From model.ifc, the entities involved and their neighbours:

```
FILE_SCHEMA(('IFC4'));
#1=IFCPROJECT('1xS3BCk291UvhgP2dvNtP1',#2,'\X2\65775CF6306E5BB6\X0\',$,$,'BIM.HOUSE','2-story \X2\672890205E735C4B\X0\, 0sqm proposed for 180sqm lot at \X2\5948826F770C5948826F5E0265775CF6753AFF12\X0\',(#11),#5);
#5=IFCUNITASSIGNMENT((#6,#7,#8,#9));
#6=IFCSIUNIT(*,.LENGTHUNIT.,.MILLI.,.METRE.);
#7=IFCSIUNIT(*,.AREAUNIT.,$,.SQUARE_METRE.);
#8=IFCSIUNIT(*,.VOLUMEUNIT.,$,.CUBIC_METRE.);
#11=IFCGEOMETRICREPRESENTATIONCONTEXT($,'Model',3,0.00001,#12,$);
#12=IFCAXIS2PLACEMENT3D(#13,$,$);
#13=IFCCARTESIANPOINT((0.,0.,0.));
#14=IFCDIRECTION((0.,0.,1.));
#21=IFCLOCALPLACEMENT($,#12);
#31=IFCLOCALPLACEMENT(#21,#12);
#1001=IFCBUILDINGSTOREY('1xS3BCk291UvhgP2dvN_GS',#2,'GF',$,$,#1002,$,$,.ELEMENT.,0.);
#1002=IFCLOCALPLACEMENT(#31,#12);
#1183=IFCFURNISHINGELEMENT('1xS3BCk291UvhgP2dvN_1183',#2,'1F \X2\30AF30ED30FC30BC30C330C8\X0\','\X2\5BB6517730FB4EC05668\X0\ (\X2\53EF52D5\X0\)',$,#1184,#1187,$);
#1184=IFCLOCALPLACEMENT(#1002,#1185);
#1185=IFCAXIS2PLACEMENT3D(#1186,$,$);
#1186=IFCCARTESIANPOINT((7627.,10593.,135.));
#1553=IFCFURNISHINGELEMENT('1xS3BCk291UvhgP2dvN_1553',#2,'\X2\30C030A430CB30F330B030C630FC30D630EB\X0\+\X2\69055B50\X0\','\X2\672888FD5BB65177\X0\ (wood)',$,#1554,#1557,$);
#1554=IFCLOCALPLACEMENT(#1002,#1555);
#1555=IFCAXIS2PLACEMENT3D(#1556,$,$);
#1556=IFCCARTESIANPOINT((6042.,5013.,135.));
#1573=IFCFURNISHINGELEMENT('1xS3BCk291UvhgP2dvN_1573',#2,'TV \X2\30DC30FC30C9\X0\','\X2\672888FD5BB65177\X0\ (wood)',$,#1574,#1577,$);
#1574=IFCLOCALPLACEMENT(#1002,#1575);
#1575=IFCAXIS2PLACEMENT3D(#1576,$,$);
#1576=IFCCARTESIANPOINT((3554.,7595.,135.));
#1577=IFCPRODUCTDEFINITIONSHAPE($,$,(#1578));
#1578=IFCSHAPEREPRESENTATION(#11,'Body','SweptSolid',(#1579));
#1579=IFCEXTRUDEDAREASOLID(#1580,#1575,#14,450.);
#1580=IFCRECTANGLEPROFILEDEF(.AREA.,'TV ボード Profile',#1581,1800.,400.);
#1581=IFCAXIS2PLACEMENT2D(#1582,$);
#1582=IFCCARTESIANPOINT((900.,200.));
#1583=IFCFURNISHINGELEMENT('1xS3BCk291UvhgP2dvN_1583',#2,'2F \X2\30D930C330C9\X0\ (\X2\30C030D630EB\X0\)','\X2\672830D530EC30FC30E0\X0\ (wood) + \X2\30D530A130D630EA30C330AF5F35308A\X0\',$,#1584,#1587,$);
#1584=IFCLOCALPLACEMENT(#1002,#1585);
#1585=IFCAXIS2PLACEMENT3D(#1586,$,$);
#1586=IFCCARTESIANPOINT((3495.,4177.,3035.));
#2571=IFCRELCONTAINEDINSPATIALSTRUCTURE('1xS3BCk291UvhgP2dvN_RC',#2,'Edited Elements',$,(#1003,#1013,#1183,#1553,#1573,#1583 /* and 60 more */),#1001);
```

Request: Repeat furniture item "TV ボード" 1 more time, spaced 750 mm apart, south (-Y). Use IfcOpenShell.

```python
import numpy as np
import ifcopenshell
import ifcopenshell.api.geometry
import ifcopenshell.api.root
import ifcopenshell.util.element
import ifcopenshell.util.placement

model = ifcopenshell.open("model.ifc")


def reuse_history(source, copy):
    """copy_class also copies each property set's owner history, people and application; keep the originals."""
    for rel in copy.IsDefinedBy:
        if rel.is_a("IfcRelDefinesByProperties") and (history := rel.RelatingPropertyDefinition.OwnerHistory):
            rel.RelatingPropertyDefinition.OwnerHistory = source.OwnerHistory
            ifcopenshell.util.element.remove_deep2(model, history)


source = model.by_guid("1xS3BCk291UvhgP2dvN_1573")
base = ifcopenshell.util.placement.get_local_placement(source.ObjectPlacement)
step = np.array([0.0, -1.0, 0.0]) * 750.0

for i in range(1, 2):
    copy = ifcopenshell.api.root.copy_class(model, product=source)
    copy.Representation = ifcopenshell.util.element.copy_deep(
        model, source.Representation, exclude=["IfcGeometricRepresentationContext", "IfcRepresentationMap"]
    )
    reuse_history(source, copy)
    matrix = base.copy()
    matrix[:3, 3] += i * step
    print("added at", matrix[:3, 3].round(3) + 0.0)
    ifcopenshell.api.geometry.edit_object_placement(model, product=copy, matrix=matrix, is_si=False)

model.write("model_rev.ifc")
```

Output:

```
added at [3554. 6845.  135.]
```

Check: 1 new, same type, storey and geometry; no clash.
